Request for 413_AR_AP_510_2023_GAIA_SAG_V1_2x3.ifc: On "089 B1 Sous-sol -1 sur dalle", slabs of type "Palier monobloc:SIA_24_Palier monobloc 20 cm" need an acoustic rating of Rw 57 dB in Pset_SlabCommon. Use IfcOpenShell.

First a look at what the model holds.

```python
import ifcopenshell
import ifcopenshell.util.element

model = ifcopenshell.open("413_AR_AP_510_2023_GAIA_SAG_V1_2x3.ifc")
print(model.schema)
storey = next(s for s in model.by_type("IfcBuildingStorey") if s.Name == "089 B1 Sous-sol -1 sur dalle")
slabs = [e for e in ifcopenshell.util.element.get_decomposition(storey) if e.is_a("IfcSlab")]
seen = {}
for e in slabs:
    element_type = ifcopenshell.util.element.get_type(e)
    key = (element_type.Name if element_type != e and element_type else None, ifcopenshell.util.element.get_pset(e, "Pset_SlabCommon", "AcousticRating"))
    seen[key] = seen.get(key, 0) + 1
for (name, value), count in sorted(seen.items(), key=str):
    print(count, "x", name, "|", value)
```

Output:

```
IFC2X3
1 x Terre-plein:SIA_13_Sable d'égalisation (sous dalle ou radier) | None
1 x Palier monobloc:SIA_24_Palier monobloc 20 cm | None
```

```python
import ifcopenshell
import ifcopenshell.api.pset
import ifcopenshell.util.element

model = ifcopenshell.open("413_AR_AP_510_2023_GAIA_SAG_V1_2x3.ifc")

storey = next(s for s in model.by_type("IfcBuildingStorey") if s.Name == "089 B1 Sous-sol -1 sur dalle")
slabs = [e for e in ifcopenshell.util.element.get_decomposition(storey) if e.is_a("IfcSlab")]

count = 0
for e in slabs:
    element_type = ifcopenshell.util.element.get_type(e)
    if element_type in (None, e) or element_type.Name != "Palier monobloc:SIA_24_Palier monobloc 20 cm":
        continue
    # add_pset returns the element's existing set when there is one.
    pset = ifcopenshell.api.pset.add_pset(model, product=e, name="Pset_SlabCommon")
    ifcopenshell.api.pset.edit_pset(model, pset=pset, properties={"AcousticRating": "Rw 57 dB"})
    count += 1

print(count, "slabs updated")

model.write("413_AR_AP_510_2023_GAIA_SAG_V1_2x3_rev.ifc")
```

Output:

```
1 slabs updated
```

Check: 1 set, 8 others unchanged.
